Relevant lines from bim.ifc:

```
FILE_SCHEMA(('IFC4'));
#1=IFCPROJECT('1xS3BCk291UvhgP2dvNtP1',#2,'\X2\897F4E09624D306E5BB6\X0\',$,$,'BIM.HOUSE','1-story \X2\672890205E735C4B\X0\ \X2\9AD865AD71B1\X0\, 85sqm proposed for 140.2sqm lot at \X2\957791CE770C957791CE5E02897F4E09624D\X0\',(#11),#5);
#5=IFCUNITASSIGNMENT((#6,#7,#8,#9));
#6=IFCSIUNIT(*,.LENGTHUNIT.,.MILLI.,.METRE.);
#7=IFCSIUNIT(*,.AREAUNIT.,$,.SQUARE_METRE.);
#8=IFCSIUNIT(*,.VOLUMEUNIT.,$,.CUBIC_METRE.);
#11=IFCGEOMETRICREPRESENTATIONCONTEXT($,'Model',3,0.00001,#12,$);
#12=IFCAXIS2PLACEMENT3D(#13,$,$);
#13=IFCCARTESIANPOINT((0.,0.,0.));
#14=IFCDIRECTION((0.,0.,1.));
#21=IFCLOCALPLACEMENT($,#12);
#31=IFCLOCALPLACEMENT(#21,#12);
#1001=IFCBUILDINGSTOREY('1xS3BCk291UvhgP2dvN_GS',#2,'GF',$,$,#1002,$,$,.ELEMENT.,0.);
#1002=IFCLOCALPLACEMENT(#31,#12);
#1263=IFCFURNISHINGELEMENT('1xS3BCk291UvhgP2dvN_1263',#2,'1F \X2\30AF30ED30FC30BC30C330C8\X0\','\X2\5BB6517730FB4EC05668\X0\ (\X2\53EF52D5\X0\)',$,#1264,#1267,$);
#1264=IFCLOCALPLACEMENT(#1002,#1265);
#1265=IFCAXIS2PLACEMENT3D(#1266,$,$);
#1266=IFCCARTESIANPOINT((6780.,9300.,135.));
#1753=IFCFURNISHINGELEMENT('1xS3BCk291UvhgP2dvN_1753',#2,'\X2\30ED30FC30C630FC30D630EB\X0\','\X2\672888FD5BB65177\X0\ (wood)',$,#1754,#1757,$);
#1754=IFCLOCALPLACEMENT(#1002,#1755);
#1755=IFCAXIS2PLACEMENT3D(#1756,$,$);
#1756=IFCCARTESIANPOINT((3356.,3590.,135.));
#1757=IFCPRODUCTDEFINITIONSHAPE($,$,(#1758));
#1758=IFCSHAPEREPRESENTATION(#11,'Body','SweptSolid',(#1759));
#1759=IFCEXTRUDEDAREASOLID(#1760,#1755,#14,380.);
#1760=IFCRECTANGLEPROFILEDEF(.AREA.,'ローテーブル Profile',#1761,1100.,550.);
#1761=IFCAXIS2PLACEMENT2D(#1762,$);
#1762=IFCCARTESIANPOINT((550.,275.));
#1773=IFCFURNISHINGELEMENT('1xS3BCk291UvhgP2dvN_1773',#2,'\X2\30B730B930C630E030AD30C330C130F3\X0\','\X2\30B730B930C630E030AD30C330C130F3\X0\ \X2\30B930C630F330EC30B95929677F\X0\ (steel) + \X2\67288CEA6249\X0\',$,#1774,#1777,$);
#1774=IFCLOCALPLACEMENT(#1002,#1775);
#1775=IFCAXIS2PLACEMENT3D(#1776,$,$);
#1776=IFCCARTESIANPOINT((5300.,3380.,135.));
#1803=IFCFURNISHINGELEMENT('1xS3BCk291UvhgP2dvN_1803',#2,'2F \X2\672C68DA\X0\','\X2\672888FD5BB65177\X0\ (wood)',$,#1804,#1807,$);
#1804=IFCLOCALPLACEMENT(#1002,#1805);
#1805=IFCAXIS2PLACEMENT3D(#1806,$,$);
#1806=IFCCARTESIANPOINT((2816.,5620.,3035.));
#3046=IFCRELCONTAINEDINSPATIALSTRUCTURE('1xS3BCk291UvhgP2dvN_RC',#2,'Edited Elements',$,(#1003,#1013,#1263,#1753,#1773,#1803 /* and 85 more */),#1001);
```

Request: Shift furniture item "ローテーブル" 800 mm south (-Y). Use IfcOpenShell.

```python
import ifcopenshell
import ifcopenshell.api.geometry
import ifcopenshell.util.placement
import ifcopenshell.util.unit

model = ifcopenshell.open("bim.ifc")
unit_scale = ifcopenshell.util.unit.calculate_unit_scale(model)

item = model.by_guid("1xS3BCk291UvhgP2dvN_1753")
matrix = ifcopenshell.util.placement.get_local_placement(item.ObjectPlacement)
matrix[1, 3] -= 0.8 / unit_scale
ifcopenshell.api.geometry.edit_object_placement(model, product=item, matrix=matrix, is_si=False)

print(ifcopenshell.util.placement.get_local_placement(item.ObjectPlacement).round(3) + 0.0)

model.write("bim_rev.ifc")
```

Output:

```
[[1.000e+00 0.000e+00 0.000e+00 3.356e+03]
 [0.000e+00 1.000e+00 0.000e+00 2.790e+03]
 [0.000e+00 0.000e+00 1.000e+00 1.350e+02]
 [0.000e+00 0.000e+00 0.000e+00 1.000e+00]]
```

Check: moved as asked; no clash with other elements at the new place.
